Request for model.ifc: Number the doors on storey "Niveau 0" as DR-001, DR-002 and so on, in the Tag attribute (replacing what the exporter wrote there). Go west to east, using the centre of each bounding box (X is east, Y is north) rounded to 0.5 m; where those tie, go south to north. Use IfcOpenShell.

First a look at what the model holds.

```python
import ifcopenshell
import ifcopenshell.util.element
import ifcopenshell.util.placement

model = ifcopenshell.open("model.ifc")
print(model.schema)
storey = next(s for s in model.by_type("IfcBuildingStorey") if s.Name == "Niveau 0")
doors = [e for e in ifcopenshell.util.element.get_decomposition(storey) if e.is_a("IfcDoor")]
for e in sorted(doors, key=lambda e: e.id()):
    origin = ifcopenshell.util.placement.get_local_placement(e.ObjectPlacement)[:3, 3]
    print(e.id(), e.Tag, e.Name, origin.round(2) + 0.0, sep=" | ")
```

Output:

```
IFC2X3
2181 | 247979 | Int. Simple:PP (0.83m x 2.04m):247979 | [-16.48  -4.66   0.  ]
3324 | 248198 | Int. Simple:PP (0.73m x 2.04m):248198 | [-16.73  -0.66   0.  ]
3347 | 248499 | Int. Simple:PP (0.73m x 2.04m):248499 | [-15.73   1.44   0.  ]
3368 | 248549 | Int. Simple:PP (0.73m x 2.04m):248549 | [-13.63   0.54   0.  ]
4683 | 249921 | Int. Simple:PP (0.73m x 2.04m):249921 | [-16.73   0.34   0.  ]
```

```python
import ifcopenshell
import ifcopenshell.geom
import ifcopenshell.util.element
import ifcopenshell.util.shape

model = ifcopenshell.open("model.ifc")
settings = ifcopenshell.geom.settings()
settings.set("use-world-coords", True)


def centre(element):
    shape = ifcopenshell.geom.create_shape(settings, element)
    return ifcopenshell.util.shape.get_bbox_centroid(shape.geometry)


storey = next(s for s in model.by_type("IfcBuildingStorey") if s.Name == "Niveau 0")
doors = [e for e in ifcopenshell.util.element.get_decomposition(storey) if e.is_a("IfcDoor")]

# Insertion points can sit at a corner or the storey origin, so sort by the geometry (in metres).
centres = {e: centre(e) for e in doors}
doors.sort(key=lambda e: (round(centres[e][0] / 0.5), centres[e][1]))

for i, e in enumerate(doors, start=1):
    number = f"DR-0{i:02d}"
    e.Tag = number
    print(e.id(), number)

model.write("model_updated.ifc")
```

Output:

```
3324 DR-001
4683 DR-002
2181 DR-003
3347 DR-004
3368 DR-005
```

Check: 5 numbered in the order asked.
